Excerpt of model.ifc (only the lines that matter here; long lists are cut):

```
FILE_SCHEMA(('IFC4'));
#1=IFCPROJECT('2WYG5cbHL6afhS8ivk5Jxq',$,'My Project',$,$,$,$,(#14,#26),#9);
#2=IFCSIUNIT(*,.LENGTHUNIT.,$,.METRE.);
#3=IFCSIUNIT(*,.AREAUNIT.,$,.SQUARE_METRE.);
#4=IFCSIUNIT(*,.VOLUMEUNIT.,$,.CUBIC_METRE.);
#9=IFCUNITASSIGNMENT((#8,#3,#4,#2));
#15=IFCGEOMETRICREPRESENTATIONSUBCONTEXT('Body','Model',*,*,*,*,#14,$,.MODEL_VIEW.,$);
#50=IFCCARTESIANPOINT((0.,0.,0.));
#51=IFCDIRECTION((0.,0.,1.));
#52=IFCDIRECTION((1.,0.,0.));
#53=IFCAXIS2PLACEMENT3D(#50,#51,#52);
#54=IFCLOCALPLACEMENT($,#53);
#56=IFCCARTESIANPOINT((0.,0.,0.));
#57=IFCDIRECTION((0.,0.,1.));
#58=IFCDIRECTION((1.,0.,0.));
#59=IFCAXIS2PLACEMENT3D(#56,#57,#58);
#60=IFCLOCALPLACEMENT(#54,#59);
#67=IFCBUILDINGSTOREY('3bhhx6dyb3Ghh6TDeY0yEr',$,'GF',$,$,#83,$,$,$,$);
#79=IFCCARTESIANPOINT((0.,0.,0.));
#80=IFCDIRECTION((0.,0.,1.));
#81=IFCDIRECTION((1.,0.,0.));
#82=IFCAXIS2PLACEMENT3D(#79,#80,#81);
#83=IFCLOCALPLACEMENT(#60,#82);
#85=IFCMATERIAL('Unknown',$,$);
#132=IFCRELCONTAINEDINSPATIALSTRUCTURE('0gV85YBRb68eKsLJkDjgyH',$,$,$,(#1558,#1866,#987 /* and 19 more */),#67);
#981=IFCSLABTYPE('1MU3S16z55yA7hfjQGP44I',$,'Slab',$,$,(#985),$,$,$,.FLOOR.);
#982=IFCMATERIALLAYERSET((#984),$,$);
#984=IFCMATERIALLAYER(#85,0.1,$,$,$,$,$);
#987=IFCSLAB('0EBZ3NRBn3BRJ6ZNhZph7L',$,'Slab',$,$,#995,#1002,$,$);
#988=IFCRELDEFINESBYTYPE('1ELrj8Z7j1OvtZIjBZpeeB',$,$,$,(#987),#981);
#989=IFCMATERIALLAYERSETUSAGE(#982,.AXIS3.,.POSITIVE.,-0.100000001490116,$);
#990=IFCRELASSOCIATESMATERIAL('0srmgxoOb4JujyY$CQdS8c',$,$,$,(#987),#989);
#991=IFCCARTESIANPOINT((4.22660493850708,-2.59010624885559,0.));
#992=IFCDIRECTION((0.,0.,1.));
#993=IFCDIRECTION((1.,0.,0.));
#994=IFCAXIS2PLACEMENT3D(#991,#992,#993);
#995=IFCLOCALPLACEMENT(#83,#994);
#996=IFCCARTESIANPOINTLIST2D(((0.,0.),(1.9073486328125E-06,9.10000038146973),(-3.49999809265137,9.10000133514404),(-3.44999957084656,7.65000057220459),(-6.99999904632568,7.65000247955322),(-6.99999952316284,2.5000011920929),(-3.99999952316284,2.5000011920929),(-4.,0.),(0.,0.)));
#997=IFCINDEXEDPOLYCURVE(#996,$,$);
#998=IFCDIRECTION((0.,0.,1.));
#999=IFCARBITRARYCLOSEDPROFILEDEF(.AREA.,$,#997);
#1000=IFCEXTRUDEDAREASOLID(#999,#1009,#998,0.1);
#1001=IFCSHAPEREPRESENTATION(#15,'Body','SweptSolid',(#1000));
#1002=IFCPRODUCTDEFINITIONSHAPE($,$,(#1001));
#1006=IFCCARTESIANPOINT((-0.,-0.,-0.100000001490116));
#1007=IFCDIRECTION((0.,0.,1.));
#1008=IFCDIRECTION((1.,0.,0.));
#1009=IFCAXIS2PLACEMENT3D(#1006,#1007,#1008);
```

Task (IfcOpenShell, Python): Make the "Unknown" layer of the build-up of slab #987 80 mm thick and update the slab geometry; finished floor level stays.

```python
import ifcopenshell
import ifcopenshell.util.element
import ifcopenshell.util.representation

model = ifcopenshell.open("model.ifc")

layer_set = model.by_id(982)
layer = next(l for l in layer_set.MaterialLayers if l.Material and l.Material.Name == "Unknown")
change = 0.08 - layer.LayerThickness
layer.LayerThickness += change

# Geometry does not follow the layer set by itself.
slabs = [e for e in ifcopenshell.util.element.get_elements_by_material(model, layer_set) if e.is_a("IfcSlab")]
for slab in sorted(slabs, key=lambda e: e.id()):
    body = ifcopenshell.util.representation.get_representation(slab, "Model", "Body")
    solid = body.Items[0]
    old_depth = solid.Depth
    solid.Depth += change
    # Extruded upwards: lower the start of the extrusion so the top stays.
    x, y, z = solid.Position.Location.Coordinates
    solid.Position.Location = model.createIfcCartesianPoint((x, y, z - change))
    print(slab.id(), f"{old_depth:g} -> {solid.Depth:g}")

# The layers are counted up from the underside, which has moved.
for usage in {ifcopenshell.util.element.get_material(slab) for slab in slabs}:
    usage.OffsetFromReferenceLine -= change

model.write("model_v2.ifc")
```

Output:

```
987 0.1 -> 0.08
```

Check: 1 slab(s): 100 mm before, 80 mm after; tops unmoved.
